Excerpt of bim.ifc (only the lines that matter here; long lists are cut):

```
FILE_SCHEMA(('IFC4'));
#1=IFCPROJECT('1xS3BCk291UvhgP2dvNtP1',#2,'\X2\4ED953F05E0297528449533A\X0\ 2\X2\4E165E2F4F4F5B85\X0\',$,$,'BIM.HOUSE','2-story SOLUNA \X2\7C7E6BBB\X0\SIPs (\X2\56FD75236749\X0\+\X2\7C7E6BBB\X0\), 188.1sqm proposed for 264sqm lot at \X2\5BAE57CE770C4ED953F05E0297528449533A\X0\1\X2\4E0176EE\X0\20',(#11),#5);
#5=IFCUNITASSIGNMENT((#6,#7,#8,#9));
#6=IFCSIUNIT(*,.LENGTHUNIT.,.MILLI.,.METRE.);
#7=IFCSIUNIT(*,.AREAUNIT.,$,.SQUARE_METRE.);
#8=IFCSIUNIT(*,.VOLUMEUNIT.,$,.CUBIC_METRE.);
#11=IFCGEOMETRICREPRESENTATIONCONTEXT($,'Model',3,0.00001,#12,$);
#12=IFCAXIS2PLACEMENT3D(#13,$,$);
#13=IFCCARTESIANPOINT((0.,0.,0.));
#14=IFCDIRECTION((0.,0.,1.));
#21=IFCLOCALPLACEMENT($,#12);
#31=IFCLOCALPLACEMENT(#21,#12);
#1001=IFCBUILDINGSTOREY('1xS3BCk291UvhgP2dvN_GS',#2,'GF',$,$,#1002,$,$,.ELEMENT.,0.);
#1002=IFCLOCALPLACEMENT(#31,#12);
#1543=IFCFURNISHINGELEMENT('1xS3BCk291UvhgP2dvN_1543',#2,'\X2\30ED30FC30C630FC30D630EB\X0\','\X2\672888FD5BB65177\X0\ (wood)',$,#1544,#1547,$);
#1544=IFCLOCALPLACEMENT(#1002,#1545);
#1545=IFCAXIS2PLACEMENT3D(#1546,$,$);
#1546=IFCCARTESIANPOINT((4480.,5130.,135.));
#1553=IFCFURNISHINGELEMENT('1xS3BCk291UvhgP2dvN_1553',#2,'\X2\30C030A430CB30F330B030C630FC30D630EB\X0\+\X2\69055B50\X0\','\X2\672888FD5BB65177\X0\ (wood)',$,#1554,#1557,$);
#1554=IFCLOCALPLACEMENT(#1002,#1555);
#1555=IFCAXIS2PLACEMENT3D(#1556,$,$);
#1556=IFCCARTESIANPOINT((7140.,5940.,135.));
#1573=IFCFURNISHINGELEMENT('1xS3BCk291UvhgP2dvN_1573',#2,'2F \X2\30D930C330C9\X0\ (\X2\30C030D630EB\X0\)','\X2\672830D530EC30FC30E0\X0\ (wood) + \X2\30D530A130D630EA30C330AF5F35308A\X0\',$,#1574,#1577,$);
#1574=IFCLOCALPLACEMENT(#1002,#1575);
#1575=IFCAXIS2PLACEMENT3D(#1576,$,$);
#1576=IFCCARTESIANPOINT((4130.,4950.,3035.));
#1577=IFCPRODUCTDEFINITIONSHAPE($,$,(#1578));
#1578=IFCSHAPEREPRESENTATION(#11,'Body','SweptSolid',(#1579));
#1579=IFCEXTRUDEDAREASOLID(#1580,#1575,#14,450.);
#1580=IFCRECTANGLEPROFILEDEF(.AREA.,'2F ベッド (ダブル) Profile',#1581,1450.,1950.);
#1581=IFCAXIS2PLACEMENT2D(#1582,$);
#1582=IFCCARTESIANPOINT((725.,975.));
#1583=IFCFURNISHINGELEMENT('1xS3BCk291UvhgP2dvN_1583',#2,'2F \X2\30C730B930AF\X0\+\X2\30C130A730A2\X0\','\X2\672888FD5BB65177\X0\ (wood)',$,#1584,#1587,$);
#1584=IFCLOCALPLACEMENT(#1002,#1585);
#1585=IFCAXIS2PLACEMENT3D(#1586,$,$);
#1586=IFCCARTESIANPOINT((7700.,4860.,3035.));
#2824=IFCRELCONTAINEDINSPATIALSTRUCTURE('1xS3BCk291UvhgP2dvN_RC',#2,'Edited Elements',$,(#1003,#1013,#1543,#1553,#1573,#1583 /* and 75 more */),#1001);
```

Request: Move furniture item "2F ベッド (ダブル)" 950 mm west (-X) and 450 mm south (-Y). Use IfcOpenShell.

```python
import ifcopenshell
import ifcopenshell.api.geometry
import ifcopenshell.util.placement
import ifcopenshell.util.unit

model = ifcopenshell.open("bim.ifc")
unit_scale = ifcopenshell.util.unit.calculate_unit_scale(model)

item = model.by_id(1573)
matrix = ifcopenshell.util.placement.get_local_placement(item.ObjectPlacement)
matrix[0, 3] -= 0.95 / unit_scale
matrix[1, 3] -= 0.45 / unit_scale
ifcopenshell.api.geometry.edit_object_placement(model, product=item, matrix=matrix, is_si=False)

print(ifcopenshell.util.placement.get_local_placement(item.ObjectPlacement).round(3) + 0.0)

model.write("bim_rev.ifc")
```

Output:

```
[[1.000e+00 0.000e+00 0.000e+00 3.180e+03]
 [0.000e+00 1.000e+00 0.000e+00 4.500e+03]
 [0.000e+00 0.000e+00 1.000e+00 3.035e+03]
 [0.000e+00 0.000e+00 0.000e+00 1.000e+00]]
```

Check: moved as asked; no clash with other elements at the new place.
